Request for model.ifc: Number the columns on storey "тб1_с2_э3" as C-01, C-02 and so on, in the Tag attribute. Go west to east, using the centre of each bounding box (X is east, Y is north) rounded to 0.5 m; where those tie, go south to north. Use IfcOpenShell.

First a look at what the model holds.

```python
import ifcopenshell
import ifcopenshell.util.element
import ifcopenshell.util.placement

model = ifcopenshell.open("model.ifc")
print(model.schema)
storey = next(s for s in model.by_type("IfcBuildingStorey") if s.Name == "тб1_с2_э3")
columns = [e for e in ifcopenshell.util.element.get_decomposition(storey) if e.is_a("IfcColumn")]
for e in sorted(columns, key=lambda e: e.id()):
    origin = ifcopenshell.util.placement.get_local_placement(e.ObjectPlacement)[:3, 3]
    print(e.id(), e.Tag, e.Name, origin.round(2) + 0.0, sep=" | ")
```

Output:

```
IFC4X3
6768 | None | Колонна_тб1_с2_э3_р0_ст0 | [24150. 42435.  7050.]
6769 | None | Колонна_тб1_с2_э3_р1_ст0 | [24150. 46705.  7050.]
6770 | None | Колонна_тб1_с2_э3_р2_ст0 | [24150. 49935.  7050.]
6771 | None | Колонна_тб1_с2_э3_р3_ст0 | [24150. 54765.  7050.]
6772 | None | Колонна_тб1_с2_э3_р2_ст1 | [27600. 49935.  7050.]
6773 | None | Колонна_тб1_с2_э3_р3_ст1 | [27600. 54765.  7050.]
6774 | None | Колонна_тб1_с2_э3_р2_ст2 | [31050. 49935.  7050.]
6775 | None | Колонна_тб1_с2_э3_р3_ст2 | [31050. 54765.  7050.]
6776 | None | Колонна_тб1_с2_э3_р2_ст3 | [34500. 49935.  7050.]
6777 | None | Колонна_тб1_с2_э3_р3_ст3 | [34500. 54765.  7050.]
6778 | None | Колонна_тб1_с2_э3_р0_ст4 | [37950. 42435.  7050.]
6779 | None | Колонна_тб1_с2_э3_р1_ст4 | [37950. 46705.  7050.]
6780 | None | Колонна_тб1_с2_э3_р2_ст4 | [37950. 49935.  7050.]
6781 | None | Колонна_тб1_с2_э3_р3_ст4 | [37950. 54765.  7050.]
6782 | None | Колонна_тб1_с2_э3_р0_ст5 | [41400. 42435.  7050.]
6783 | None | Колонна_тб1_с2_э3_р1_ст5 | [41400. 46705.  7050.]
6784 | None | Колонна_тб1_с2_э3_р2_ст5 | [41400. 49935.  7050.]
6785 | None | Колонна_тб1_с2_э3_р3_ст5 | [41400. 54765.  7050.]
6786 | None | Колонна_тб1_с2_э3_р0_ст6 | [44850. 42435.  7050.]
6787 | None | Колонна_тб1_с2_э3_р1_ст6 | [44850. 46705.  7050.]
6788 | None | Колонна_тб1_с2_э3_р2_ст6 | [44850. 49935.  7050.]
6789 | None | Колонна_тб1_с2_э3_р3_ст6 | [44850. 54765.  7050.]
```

```python
import ifcopenshell
import ifcopenshell.geom
import ifcopenshell.util.element
import ifcopenshell.util.shape

model = ifcopenshell.open("model.ifc")
settings = ifcopenshell.geom.settings()
settings.set("use-world-coords", True)


def centre(element):
    shape = ifcopenshell.geom.create_shape(settings, element)
    return ifcopenshell.util.shape.get_bbox_centroid(shape.geometry)


storey = next(s for s in model.by_type("IfcBuildingStorey") if s.Name == "тб1_с2_э3")
columns = [e for e in ifcopenshell.util.element.get_decomposition(storey) if e.is_a("IfcColumn")]

# Insertion points can sit at a corner or the storey origin, so sort by the geometry (in metres).
centres = {e: centre(e) for e in columns}
columns.sort(key=lambda e: (round(centres[e][0] / 0.5), centres[e][1]))

for i, e in enumerate(columns, start=1):
    number = f"C-{i:02d}"
    e.Tag = number
    print(e.id(), number)

model.write("model-out.ifc")
```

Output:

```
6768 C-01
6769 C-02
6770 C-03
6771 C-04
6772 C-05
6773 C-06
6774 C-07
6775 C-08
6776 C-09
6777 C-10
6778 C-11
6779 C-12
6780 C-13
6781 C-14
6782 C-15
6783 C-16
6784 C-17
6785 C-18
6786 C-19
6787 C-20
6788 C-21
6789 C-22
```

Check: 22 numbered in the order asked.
